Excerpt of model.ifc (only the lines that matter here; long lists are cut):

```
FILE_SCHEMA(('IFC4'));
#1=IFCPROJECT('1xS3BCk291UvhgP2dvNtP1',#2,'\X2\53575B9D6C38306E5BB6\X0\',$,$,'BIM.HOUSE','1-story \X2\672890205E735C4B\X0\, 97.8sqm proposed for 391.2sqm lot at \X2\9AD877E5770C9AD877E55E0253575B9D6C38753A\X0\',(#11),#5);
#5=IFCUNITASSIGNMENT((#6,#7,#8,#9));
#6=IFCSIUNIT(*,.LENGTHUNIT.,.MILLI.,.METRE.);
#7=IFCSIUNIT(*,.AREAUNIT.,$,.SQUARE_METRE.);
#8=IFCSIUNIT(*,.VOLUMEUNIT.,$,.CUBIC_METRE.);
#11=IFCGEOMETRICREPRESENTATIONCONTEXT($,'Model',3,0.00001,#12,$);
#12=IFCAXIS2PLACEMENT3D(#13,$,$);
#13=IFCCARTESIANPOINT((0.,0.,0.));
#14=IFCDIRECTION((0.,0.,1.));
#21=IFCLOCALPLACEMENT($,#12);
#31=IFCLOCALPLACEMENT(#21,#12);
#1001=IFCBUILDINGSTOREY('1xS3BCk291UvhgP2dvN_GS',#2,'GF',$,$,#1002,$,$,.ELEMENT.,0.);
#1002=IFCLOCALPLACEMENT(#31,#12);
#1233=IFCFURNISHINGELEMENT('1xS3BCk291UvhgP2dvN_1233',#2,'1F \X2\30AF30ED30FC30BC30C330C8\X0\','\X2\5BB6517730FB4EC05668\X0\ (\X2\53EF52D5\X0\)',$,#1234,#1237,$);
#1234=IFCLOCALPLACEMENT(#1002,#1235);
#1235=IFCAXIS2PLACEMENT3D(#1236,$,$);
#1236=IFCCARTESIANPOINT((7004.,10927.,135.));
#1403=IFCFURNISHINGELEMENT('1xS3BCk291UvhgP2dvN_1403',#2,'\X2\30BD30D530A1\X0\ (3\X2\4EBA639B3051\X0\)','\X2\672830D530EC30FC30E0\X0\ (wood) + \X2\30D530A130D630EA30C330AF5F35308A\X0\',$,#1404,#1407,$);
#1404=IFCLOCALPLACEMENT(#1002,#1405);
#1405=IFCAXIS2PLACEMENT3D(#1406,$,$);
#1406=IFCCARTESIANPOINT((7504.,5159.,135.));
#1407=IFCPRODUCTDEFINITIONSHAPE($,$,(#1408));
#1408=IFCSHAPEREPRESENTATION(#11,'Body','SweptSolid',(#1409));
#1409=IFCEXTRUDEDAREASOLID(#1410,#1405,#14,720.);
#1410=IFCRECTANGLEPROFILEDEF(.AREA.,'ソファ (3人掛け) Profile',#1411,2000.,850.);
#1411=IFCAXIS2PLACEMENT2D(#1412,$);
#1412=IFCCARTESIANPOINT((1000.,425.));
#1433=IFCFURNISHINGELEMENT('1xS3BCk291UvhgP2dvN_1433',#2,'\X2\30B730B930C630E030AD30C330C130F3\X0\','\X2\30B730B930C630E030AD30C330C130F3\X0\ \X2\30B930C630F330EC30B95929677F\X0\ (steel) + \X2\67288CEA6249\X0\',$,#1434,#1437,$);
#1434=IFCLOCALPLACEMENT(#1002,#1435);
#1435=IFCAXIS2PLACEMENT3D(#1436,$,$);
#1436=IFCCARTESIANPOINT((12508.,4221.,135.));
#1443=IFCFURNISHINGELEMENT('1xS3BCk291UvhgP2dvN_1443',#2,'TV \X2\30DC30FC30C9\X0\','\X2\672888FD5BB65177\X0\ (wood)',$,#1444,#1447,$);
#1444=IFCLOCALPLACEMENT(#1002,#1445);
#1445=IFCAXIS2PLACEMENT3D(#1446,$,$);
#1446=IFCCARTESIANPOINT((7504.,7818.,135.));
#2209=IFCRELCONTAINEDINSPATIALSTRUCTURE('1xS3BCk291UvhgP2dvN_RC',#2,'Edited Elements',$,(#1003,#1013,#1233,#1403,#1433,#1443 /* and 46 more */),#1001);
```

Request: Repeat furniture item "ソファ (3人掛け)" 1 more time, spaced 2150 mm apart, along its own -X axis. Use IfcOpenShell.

```python
import ifcopenshell
import ifcopenshell.api.geometry
import ifcopenshell.api.root
import ifcopenshell.util.element
import ifcopenshell.util.placement

model = ifcopenshell.open("model.ifc")


def reuse_history(source, copy):
    """copy_class also copies each property set's owner history, people and application; keep the originals."""
    for rel in copy.IsDefinedBy:
        if rel.is_a("IfcRelDefinesByProperties") and (history := rel.RelatingPropertyDefinition.OwnerHistory):
            rel.RelatingPropertyDefinition.OwnerHistory = source.OwnerHistory
            ifcopenshell.util.element.remove_deep2(model, history)


source = model.by_guid("1xS3BCk291UvhgP2dvN_1403")
base = ifcopenshell.util.placement.get_local_placement(source.ObjectPlacement)
step = -base[:3, 0] * 2150.0

for i in range(1, 2):
    copy = ifcopenshell.api.root.copy_class(model, product=source)
    copy.Representation = ifcopenshell.util.element.copy_deep(
        model, source.Representation, exclude=["IfcGeometricRepresentationContext", "IfcRepresentationMap"]
    )
    reuse_history(source, copy)
    matrix = base.copy()
    matrix[:3, 3] += i * step
    print("added at", matrix[:3, 3].round(3) + 0.0)
    ifcopenshell.api.geometry.edit_object_placement(model, product=copy, matrix=matrix, is_si=False)

model.write("model_edited.ifc")
```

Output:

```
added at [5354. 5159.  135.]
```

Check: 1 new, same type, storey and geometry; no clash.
